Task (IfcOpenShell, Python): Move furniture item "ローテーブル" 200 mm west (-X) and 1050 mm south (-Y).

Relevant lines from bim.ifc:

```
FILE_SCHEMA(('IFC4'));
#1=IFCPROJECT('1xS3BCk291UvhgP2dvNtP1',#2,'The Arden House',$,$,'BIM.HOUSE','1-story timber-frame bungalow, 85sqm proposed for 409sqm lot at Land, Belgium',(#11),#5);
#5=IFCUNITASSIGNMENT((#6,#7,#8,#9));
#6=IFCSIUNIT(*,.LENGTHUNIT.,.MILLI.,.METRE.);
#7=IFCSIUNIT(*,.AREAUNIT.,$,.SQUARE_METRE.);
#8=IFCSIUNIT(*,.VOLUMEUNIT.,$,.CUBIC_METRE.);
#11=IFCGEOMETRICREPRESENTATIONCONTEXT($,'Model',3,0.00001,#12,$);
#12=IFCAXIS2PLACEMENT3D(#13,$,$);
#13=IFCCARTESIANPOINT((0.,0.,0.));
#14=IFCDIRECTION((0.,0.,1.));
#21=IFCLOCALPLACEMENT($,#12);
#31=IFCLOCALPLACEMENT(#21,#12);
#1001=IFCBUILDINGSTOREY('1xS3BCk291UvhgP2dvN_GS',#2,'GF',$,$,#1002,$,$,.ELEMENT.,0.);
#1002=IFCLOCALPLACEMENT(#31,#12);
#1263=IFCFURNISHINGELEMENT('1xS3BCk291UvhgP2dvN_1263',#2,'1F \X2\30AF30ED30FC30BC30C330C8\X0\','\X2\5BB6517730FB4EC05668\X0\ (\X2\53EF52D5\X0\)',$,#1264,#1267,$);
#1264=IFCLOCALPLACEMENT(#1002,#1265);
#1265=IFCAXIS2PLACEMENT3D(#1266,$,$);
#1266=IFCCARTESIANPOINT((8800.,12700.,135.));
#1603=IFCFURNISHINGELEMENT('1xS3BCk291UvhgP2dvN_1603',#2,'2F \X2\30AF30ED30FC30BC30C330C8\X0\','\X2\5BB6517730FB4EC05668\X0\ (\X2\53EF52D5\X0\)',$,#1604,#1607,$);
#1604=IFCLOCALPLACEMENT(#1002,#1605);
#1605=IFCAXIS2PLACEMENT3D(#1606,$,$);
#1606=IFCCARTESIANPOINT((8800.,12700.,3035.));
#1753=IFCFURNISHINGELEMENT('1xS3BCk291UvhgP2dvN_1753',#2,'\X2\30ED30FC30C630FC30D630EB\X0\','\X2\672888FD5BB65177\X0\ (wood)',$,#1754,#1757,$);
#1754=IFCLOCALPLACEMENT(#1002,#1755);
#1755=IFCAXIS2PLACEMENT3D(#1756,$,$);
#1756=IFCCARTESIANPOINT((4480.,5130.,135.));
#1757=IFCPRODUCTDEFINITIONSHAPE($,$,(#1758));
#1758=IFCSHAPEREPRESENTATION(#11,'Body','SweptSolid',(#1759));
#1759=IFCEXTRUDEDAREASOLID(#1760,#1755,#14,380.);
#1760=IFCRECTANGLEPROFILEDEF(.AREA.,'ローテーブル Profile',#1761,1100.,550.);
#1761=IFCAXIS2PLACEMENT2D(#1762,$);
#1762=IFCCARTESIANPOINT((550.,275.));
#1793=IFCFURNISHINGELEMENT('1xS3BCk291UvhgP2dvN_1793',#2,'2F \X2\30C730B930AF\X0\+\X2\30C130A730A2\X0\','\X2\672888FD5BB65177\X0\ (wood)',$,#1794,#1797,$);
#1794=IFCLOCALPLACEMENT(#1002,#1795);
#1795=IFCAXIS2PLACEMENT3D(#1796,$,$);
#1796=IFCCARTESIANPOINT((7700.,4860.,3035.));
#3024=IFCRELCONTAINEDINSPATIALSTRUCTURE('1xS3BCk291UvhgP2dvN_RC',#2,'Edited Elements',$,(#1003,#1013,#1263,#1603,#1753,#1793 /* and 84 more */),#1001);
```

```python
import ifcopenshell
import ifcopenshell.api.geometry
import ifcopenshell.util.placement

model = ifcopenshell.open("bim.ifc")

item = model.by_id(1753)
matrix = ifcopenshell.util.placement.get_local_placement(item.ObjectPlacement)
matrix[0, 3] -= 200.0
matrix[1, 3] -= 1050.0
ifcopenshell.api.geometry.edit_object_placement(model, product=item, matrix=matrix, is_si=False)

print(ifcopenshell.util.placement.get_local_placement(item.ObjectPlacement).round(3) + 0.0)

model.write("bim-out.ifc")
```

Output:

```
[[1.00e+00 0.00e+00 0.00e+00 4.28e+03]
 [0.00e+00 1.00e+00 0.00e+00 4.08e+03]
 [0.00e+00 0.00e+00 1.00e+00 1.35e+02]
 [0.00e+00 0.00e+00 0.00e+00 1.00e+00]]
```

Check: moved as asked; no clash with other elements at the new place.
